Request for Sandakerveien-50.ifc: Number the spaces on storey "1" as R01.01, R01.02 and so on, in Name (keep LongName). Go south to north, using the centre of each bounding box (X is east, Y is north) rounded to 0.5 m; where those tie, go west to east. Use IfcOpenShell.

First a look at what the model holds.

```python
import ifcopenshell
import ifcopenshell.util.element
import ifcopenshell.util.placement

model = ifcopenshell.open("Sandakerveien-50.ifc")
print(model.schema)
storey = next(s for s in model.by_type("IfcBuildingStorey") if s.Name == "1")
spaces = [e for e in ifcopenshell.util.element.get_decomposition(storey) if e.is_a("IfcSpace")]
for e in sorted(spaces, key=lambda e: e.id()):
    origin = ifcopenshell.util.placement.get_local_placement(e.ObjectPlacement)[:3, 3]
    print(e.id(), e.Name, e.LongName, origin.round(2) + 0.0, sep=" | ")
```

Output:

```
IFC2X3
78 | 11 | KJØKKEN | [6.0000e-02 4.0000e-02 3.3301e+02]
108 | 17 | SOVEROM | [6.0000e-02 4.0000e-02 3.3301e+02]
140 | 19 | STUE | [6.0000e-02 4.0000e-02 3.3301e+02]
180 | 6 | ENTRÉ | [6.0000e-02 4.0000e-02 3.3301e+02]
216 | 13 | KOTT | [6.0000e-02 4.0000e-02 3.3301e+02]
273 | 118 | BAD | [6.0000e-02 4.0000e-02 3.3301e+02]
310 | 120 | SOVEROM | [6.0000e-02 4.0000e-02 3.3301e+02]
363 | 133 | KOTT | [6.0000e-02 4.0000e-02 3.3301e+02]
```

```python
import ifcopenshell
import ifcopenshell.geom
import ifcopenshell.util.element
import ifcopenshell.util.shape

model = ifcopenshell.open("Sandakerveien-50.ifc")
settings = ifcopenshell.geom.settings()
settings.set("use-world-coords", True)


def centre(element):
    shape = ifcopenshell.geom.create_shape(settings, element)
    return ifcopenshell.util.shape.get_bbox_centroid(shape.geometry)


storey = next(s for s in model.by_type("IfcBuildingStorey") if s.Name == "1")
spaces = [e for e in ifcopenshell.util.element.get_decomposition(storey) if e.is_a("IfcSpace")]

# Insertion points can sit at a corner or the storey origin, so sort by the geometry (in metres).
centres = {e: centre(e) for e in spaces}
spaces.sort(key=lambda e: (round(centres[e][1] / 0.5), centres[e][0]))

for i, e in enumerate(spaces, start=1):
    number = f"R01.{i:02d}"
    e.Name = number
    print(e.id(), number)

model.write("Sandakerveien-50_v2.ifc")
```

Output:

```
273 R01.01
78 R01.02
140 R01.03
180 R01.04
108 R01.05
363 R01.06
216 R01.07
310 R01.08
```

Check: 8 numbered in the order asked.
